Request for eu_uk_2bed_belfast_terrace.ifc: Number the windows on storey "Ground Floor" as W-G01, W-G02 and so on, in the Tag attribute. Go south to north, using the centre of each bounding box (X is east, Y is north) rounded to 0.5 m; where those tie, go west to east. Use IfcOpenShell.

First a look at what the model holds.

```python
import ifcopenshell
import ifcopenshell.util.element
import ifcopenshell.util.placement

model = ifcopenshell.open("eu_uk_2bed_belfast_terrace.ifc")
print(model.schema)
storey = next(s for s in model.by_type("IfcBuildingStorey") if s.Name == "Ground Floor")
windows = [e for e in ifcopenshell.util.element.get_decomposition(storey) if e.is_a("IfcWindow")]
for e in sorted(windows, key=lambda e: e.id()):
    origin = ifcopenshell.util.placement.get_local_placement(e.ObjectPlacement)[:3, 3]
    print(e.id(), e.Tag, e.Name, origin.round(2) + 0.0, sep=" | ")
```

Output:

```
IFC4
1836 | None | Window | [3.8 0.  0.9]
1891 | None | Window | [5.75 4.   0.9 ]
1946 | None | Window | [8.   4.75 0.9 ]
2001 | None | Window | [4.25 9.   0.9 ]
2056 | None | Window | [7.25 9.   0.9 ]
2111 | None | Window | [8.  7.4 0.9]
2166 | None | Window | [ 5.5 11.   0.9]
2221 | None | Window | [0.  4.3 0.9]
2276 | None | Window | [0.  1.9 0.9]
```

```python
import ifcopenshell
import ifcopenshell.geom
import ifcopenshell.util.element
import ifcopenshell.util.shape

model = ifcopenshell.open("eu_uk_2bed_belfast_terrace.ifc")
settings = ifcopenshell.geom.settings()
settings.set("use-world-coords", True)


def centre(element):
    shape = ifcopenshell.geom.create_shape(settings, element)
    return ifcopenshell.util.shape.get_bbox_centroid(shape.geometry)


storey = next(s for s in model.by_type("IfcBuildingStorey") if s.Name == "Ground Floor")
windows = [e for e in ifcopenshell.util.element.get_decomposition(storey) if e.is_a("IfcWindow")]

# Insertion points can sit at a corner or the storey origin, so sort by the geometry (in metres).
centres = {e: centre(e) for e in windows}
windows.sort(key=lambda e: (round(centres[e][1] / 0.5), centres[e][0]))

for i, e in enumerate(windows, start=1):
    number = f"W-G{i:02d}"
    e.Tag = number
    print(e.id(), number)

model.write("eu_uk_2bed_belfast_terrace_updated.ifc")
```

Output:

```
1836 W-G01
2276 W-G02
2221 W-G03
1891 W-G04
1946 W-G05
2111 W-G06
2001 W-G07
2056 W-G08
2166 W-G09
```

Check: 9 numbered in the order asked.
